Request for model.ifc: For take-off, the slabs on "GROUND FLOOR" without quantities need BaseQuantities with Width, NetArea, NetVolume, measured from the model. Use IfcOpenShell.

First a look at what the model holds.

```python
import ifcopenshell
import ifcopenshell.util.element
import ifcopenshell.util.unit

model = ifcopenshell.open("model.ifc")
print(model.schema)
for unit_type in ("LENGTHUNIT", "AREAUNIT", "VOLUMEUNIT"):
    print(unit_type, ifcopenshell.util.unit.calculate_unit_scale(model, unit_type))
storey = next(s for s in model.by_type("IfcBuildingStorey") if s.Name == "GROUND FLOOR")
slabs = [e for e in ifcopenshell.util.element.get_decomposition(storey) if e.is_a("IfcSlab")]
for e in sorted(slabs, key=lambda e: e.id()):
    print(e.id(), e.is_a(), e.Name, list(ifcopenshell.util.element.get_psets(e, qtos_only=True)), sep=" | ")
```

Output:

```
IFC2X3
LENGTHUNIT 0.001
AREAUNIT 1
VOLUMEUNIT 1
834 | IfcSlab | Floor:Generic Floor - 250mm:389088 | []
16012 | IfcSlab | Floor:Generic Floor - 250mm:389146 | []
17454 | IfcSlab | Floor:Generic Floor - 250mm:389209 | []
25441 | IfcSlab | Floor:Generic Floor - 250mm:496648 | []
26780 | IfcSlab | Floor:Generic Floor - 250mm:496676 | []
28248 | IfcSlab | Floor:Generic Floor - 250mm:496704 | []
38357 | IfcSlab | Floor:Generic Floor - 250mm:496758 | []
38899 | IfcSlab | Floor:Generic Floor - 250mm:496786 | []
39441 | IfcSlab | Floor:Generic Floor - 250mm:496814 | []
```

```python
import ifcopenshell
import ifcopenshell.api.pset
import ifcopenshell.geom
import ifcopenshell.util.element
import ifcopenshell.util.shape
import ifcopenshell.util.unit

model = ifcopenshell.open("model.ifc")
unit_scale = ifcopenshell.util.unit.calculate_unit_scale(model)
area_scale = ifcopenshell.util.unit.calculate_unit_scale(model, "AREAUNIT")
volume_scale = ifcopenshell.util.unit.calculate_unit_scale(model, "VOLUMEUNIT")
settings = ifcopenshell.geom.settings()

storey = next(s for s in model.by_type("IfcBuildingStorey") if s.Name == "GROUND FLOOR")
slabs = [e for e in ifcopenshell.util.element.get_decomposition(storey) if e.is_a("IfcSlab")]

for e in sorted(slabs, key=lambda e: e.id()):
    if ifcopenshell.util.element.get_psets(e, qtos_only=True, should_inherit=False):
        continue
    # Geometry comes back in metres, in the element's own axes.
    shape = ifcopenshell.geom.create_shape(settings, e)
    values = {
        "Width": ifcopenshell.util.shape.get_z(shape.geometry) / unit_scale,
        "NetArea": ifcopenshell.util.shape.get_footprint_area(shape.geometry) / area_scale,
        "NetVolume": ifcopenshell.util.shape.get_volume(shape.geometry) / volume_scale,
    }
    qto = ifcopenshell.api.pset.add_qto(model, product=e, name="BaseQuantities")
    ifcopenshell.api.pset.edit_qto(model, qto=qto, properties=values)
    print(e.id(), {k: round(v, 3) for k, v in values.items()})

model.write("model-out.ifc")
```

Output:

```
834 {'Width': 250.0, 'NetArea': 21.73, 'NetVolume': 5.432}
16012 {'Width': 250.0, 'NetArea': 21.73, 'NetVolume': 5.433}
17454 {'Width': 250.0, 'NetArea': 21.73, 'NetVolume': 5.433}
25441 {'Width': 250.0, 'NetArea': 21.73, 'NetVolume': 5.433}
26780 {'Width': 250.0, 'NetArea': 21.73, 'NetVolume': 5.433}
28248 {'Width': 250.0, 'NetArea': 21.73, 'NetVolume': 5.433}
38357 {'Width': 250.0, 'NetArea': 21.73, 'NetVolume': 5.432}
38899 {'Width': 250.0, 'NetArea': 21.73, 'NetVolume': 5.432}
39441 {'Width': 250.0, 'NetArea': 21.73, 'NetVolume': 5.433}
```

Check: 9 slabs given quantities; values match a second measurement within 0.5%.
